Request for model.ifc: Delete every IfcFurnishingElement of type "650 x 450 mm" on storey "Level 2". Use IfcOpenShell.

First a look at what the model holds.

```python
import ifcopenshell
import ifcopenshell.util.element

model = ifcopenshell.open("model.ifc")
print(model.schema)
storey = next(s for s in model.by_type("IfcBuildingStorey") if s.Name == "Level 2")
furniture = [e for e in ifcopenshell.util.element.get_decomposition(storey) if e.is_a("IfcFurnishingElement")]
seen = {}
for e in furniture:
    element_type = ifcopenshell.util.element.get_type(e)
    name = element_type.Name if element_type not in (None, e) else None
    seen[name] = seen.get(name, 0) + 1
for name, count in sorted(seen.items(), key=str):
    print(count, "x", name)
```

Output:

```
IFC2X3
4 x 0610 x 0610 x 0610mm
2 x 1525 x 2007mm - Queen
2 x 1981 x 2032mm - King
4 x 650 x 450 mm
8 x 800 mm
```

```python
import ifcopenshell
import ifcopenshell.api.root
import ifcopenshell.util.element

model = ifcopenshell.open("model.ifc")

storey = next(s for s in model.by_type("IfcBuildingStorey") if s.Name == "Level 2")
furniture = [e for e in ifcopenshell.util.element.get_decomposition(storey) if e.is_a("IfcFurnishingElement")]
targets = [e for e in furniture if (t := ifcopenshell.util.element.get_type(e)) not in (None, e) and t.Name == "650 x 450 mm"]

for e in targets:
    ifcopenshell.api.root.remove_product(model, product=e)
print(len(targets), "removed")

model.write("model_rev.ifc")
```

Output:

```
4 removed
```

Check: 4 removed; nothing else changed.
